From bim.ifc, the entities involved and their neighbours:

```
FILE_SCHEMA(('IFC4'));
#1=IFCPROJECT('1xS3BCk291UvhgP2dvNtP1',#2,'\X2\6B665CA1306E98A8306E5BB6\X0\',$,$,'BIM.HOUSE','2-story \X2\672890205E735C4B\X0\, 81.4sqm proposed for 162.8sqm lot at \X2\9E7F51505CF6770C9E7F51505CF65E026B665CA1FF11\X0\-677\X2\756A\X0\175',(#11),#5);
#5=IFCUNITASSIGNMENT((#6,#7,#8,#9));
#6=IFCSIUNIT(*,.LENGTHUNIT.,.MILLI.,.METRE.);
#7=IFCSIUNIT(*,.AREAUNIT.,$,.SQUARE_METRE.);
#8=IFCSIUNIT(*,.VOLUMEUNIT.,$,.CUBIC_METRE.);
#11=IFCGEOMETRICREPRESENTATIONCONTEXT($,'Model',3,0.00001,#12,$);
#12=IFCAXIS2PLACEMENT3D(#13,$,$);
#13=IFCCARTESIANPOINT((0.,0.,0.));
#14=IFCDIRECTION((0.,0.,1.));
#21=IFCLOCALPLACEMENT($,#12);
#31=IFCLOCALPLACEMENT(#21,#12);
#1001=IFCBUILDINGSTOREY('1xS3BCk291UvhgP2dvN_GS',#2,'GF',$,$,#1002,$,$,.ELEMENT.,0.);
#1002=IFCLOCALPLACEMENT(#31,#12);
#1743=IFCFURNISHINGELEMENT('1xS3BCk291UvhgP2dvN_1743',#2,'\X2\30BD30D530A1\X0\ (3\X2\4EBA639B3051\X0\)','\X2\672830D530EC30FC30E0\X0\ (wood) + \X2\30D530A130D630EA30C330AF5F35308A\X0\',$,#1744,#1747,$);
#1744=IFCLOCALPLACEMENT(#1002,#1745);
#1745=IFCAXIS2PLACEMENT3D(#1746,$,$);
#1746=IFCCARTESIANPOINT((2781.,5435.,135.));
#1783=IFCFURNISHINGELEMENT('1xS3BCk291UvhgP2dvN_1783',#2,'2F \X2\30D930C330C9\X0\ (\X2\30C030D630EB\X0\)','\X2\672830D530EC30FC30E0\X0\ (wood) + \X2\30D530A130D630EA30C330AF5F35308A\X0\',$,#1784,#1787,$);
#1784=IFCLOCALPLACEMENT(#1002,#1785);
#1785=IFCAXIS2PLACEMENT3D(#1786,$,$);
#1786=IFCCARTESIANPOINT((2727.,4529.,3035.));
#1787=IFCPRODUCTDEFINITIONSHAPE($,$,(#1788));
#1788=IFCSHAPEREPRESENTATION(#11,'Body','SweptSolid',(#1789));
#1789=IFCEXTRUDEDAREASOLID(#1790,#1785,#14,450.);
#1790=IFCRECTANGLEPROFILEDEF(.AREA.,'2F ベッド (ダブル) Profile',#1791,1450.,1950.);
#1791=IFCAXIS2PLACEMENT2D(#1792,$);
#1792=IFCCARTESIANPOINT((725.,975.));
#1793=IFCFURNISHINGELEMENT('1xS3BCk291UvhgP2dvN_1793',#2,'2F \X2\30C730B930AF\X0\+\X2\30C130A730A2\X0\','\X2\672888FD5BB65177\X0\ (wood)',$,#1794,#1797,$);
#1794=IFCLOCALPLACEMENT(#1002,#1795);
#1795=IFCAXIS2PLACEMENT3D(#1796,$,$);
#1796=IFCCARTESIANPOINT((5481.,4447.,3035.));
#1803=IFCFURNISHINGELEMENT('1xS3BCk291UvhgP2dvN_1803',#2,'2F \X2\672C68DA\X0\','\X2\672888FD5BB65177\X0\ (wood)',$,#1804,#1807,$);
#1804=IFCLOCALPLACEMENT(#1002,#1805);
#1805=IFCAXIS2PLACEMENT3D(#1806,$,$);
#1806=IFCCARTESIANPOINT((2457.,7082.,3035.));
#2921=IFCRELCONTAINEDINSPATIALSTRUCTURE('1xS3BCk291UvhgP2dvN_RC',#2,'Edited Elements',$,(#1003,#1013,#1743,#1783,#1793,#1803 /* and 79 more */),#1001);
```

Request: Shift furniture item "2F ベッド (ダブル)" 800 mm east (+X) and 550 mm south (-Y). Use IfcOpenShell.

```python
import ifcopenshell
import ifcopenshell.api.geometry
import ifcopenshell.util.placement

model = ifcopenshell.open("bim.ifc")

item = model.by_guid("1xS3BCk291UvhgP2dvN_1783")
matrix = ifcopenshell.util.placement.get_local_placement(item.ObjectPlacement)
matrix[0, 3] += 800.0
matrix[1, 3] -= 550.0
ifcopenshell.api.geometry.edit_object_placement(model, product=item, matrix=matrix, is_si=False)

print(ifcopenshell.util.placement.get_local_placement(item.ObjectPlacement).round(3) + 0.0)

model.write("bim_rev.ifc")
```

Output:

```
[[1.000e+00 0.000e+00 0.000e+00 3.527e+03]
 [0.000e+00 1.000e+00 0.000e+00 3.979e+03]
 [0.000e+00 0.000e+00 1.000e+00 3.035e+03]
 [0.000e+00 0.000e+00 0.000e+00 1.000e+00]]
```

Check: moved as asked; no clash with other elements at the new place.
